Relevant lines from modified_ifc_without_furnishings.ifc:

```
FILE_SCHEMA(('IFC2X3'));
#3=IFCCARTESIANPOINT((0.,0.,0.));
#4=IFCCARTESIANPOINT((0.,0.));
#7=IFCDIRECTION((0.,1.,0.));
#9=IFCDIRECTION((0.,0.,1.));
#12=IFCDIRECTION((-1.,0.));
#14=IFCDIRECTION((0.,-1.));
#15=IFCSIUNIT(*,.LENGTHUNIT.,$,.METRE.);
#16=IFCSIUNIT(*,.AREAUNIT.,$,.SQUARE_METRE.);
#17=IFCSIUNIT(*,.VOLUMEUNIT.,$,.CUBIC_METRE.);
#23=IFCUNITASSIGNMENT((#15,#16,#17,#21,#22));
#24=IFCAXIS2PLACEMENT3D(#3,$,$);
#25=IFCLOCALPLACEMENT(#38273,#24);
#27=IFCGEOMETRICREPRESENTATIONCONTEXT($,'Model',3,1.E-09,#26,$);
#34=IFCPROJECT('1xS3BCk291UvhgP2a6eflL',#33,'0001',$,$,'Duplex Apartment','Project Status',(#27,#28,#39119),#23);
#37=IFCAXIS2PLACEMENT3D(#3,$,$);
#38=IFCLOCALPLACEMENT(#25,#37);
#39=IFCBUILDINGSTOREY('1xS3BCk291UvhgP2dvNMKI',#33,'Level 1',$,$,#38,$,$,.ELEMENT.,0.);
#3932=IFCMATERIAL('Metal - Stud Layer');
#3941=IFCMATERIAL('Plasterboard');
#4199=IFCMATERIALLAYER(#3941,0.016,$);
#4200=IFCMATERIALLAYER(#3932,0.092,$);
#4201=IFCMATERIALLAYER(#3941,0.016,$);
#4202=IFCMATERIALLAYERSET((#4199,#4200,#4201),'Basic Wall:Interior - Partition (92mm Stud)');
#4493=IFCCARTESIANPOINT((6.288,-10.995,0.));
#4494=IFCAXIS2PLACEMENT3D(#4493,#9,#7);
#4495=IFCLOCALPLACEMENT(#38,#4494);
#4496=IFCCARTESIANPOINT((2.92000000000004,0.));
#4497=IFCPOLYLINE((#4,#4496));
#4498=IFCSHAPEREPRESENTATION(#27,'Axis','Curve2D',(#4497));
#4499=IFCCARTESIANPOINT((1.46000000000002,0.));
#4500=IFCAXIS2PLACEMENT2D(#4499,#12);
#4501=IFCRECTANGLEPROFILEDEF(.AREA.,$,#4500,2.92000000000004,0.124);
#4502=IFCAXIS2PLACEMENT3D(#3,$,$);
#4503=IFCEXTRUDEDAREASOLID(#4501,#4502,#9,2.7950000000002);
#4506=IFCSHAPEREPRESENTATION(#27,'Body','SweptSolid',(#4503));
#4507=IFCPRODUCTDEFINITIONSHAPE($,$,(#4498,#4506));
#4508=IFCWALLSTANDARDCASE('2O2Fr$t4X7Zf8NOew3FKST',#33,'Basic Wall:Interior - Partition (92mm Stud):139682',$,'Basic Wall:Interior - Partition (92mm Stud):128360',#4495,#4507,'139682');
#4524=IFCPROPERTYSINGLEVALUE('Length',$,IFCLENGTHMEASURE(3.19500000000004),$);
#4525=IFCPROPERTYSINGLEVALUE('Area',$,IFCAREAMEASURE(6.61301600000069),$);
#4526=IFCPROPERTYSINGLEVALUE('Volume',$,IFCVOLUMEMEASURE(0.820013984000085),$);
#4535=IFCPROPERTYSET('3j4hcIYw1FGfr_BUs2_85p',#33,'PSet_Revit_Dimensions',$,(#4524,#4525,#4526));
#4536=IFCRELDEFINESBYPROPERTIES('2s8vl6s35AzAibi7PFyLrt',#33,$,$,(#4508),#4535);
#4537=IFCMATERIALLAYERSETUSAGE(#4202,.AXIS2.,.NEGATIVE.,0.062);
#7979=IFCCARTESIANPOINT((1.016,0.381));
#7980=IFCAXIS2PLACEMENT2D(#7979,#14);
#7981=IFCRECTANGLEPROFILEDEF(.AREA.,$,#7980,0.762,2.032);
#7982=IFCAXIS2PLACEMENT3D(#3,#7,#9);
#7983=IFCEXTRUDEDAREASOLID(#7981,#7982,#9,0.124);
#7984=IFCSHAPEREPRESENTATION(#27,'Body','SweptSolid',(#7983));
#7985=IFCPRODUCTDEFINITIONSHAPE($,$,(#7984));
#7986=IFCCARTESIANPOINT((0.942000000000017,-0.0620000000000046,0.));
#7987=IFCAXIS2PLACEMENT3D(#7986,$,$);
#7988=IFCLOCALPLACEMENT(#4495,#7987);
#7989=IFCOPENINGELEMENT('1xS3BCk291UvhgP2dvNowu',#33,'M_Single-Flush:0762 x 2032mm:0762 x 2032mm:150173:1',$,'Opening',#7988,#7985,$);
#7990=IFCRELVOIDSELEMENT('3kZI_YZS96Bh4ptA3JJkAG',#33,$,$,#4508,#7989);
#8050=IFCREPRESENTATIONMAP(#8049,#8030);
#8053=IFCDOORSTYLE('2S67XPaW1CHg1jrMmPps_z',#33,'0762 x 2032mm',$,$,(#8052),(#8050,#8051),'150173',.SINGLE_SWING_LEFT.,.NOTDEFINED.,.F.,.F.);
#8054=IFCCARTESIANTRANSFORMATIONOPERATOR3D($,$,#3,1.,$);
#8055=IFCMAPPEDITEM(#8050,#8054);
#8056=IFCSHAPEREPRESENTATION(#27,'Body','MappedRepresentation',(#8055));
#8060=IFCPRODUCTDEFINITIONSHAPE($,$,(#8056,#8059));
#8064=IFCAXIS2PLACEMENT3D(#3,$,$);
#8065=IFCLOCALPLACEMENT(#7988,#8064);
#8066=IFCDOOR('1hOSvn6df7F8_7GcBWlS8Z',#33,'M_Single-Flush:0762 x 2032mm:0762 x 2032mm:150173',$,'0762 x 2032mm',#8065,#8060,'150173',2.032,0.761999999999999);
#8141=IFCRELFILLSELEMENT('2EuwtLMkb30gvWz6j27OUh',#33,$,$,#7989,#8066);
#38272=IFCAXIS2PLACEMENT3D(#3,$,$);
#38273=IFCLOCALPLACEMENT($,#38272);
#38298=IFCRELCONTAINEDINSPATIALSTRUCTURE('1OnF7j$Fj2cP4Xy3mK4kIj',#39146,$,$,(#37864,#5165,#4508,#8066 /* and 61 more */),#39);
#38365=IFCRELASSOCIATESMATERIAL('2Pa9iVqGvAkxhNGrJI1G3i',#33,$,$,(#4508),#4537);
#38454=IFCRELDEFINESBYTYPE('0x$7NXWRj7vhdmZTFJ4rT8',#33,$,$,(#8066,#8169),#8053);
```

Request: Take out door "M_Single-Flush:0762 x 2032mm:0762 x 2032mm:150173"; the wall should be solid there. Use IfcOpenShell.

```python
import ifcopenshell
import ifcopenshell.api.feature
import ifcopenshell.api.pset
import ifcopenshell.api.root
import ifcopenshell.geom
import ifcopenshell.util.element
import ifcopenshell.util.shape
import ifcopenshell.util.unit

model = ifcopenshell.open("modified_ifc_without_furnishings.ifc")
area_scale = ifcopenshell.util.unit.calculate_unit_scale(model, "AREAUNIT")
volume_scale = ifcopenshell.util.unit.calculate_unit_scale(model, "VOLUMEUNIT")
settings = ifcopenshell.geom.settings()


def volume(element):
    """Net volume in cubic metres, openings subtracted."""
    shape = ifcopenshell.geom.create_shape(settings, element)
    return ifcopenshell.util.shape.get_volume(shape.geometry)


door = model.by_id(8066)
opening = door.FillsVoids[0].RelatingOpeningElement
wall = opening.VoidsElements[0].RelatingBuildingElement
before = volume(wall)

ifcopenshell.api.root.remove_product(model, product=door)
ifcopenshell.api.feature.remove_feature(model, feature=opening)

after = volume(wall)
thickness = 0.124  # wall thickness in metres

# Update the wall's stored quantities.
pset = model.by_id(ifcopenshell.util.element.get_pset(wall, "PSet_Revit_Dimensions", should_inherit=False)["id"])
ifcopenshell.api.pset.edit_pset(model, pset=pset, properties={
    "Area": model.create_entity("IfcAreaMeasure", after / thickness / area_scale),
    "Volume": model.create_entity("IfcVolumeMeasure", after / volume_scale),
})

print(f"wall volume {before:.3f} -> {after:.3f} m3")

model.write("modified_ifc_without_furnishings-out.ifc")
```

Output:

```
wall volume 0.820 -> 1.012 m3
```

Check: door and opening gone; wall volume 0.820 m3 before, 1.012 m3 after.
